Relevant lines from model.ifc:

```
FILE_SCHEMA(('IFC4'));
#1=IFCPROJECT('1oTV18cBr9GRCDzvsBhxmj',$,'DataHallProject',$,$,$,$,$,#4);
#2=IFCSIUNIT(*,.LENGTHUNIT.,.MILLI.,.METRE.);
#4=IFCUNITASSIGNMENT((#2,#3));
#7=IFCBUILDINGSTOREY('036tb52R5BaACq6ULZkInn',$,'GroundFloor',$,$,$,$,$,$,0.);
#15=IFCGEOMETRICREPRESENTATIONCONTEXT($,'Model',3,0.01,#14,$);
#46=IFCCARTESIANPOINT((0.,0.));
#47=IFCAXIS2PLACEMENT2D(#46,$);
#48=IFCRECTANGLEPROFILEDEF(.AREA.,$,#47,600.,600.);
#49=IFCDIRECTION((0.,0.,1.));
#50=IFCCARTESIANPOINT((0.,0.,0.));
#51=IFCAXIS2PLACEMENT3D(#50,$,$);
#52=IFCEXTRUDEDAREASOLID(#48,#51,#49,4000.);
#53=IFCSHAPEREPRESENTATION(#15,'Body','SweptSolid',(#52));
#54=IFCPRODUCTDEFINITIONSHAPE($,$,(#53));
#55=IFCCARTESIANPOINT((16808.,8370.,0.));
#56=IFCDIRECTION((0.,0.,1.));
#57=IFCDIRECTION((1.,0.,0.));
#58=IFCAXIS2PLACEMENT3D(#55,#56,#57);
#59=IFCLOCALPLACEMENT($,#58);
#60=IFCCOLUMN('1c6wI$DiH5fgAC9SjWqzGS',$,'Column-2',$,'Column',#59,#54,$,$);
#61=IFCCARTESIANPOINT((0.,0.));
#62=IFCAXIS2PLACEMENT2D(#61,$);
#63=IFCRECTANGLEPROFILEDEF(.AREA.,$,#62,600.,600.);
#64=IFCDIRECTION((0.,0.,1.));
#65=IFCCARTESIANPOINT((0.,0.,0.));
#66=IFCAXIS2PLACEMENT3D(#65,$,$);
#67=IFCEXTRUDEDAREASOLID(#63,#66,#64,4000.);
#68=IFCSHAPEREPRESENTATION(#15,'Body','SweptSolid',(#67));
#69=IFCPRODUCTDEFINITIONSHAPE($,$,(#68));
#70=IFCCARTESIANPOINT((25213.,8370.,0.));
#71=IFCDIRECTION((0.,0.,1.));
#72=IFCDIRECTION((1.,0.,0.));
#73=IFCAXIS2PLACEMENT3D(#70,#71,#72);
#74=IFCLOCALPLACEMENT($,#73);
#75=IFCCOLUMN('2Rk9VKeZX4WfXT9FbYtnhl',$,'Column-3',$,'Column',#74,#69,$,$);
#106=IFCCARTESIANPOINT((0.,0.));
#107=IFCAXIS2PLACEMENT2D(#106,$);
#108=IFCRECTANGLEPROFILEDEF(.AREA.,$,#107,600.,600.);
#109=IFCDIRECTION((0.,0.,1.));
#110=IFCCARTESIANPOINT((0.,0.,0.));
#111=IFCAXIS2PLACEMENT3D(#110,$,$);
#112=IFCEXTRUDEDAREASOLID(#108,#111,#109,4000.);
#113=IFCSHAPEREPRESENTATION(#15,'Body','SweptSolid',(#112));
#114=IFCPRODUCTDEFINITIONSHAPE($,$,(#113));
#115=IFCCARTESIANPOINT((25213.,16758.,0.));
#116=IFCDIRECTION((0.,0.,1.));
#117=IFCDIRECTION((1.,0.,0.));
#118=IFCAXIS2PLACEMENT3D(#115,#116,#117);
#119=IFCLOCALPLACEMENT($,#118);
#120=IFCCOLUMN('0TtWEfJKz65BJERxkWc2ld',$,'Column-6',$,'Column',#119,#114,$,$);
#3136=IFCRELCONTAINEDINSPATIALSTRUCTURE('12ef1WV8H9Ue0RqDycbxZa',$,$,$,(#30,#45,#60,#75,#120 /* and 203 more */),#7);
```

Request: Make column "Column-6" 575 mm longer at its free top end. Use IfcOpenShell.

```python
import ifcopenshell

model = ifcopenshell.open("model.ifc")

member = model.by_guid("0TtWEfJKz65BJERxkWc2ld")
change = 575.0

# The extrusion runs towards the end named, so only its depth changes.
body = next(r for r in member.Representation.Representations if r.RepresentationIdentifier == "Body")
solid = body.Items[0]
old_length = solid.Depth
solid.Depth += change

print(f"length {old_length:g} -> {solid.Depth:g}")

model.write("model_rev.ifc")
```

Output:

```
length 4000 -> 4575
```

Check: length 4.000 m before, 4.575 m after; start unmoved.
